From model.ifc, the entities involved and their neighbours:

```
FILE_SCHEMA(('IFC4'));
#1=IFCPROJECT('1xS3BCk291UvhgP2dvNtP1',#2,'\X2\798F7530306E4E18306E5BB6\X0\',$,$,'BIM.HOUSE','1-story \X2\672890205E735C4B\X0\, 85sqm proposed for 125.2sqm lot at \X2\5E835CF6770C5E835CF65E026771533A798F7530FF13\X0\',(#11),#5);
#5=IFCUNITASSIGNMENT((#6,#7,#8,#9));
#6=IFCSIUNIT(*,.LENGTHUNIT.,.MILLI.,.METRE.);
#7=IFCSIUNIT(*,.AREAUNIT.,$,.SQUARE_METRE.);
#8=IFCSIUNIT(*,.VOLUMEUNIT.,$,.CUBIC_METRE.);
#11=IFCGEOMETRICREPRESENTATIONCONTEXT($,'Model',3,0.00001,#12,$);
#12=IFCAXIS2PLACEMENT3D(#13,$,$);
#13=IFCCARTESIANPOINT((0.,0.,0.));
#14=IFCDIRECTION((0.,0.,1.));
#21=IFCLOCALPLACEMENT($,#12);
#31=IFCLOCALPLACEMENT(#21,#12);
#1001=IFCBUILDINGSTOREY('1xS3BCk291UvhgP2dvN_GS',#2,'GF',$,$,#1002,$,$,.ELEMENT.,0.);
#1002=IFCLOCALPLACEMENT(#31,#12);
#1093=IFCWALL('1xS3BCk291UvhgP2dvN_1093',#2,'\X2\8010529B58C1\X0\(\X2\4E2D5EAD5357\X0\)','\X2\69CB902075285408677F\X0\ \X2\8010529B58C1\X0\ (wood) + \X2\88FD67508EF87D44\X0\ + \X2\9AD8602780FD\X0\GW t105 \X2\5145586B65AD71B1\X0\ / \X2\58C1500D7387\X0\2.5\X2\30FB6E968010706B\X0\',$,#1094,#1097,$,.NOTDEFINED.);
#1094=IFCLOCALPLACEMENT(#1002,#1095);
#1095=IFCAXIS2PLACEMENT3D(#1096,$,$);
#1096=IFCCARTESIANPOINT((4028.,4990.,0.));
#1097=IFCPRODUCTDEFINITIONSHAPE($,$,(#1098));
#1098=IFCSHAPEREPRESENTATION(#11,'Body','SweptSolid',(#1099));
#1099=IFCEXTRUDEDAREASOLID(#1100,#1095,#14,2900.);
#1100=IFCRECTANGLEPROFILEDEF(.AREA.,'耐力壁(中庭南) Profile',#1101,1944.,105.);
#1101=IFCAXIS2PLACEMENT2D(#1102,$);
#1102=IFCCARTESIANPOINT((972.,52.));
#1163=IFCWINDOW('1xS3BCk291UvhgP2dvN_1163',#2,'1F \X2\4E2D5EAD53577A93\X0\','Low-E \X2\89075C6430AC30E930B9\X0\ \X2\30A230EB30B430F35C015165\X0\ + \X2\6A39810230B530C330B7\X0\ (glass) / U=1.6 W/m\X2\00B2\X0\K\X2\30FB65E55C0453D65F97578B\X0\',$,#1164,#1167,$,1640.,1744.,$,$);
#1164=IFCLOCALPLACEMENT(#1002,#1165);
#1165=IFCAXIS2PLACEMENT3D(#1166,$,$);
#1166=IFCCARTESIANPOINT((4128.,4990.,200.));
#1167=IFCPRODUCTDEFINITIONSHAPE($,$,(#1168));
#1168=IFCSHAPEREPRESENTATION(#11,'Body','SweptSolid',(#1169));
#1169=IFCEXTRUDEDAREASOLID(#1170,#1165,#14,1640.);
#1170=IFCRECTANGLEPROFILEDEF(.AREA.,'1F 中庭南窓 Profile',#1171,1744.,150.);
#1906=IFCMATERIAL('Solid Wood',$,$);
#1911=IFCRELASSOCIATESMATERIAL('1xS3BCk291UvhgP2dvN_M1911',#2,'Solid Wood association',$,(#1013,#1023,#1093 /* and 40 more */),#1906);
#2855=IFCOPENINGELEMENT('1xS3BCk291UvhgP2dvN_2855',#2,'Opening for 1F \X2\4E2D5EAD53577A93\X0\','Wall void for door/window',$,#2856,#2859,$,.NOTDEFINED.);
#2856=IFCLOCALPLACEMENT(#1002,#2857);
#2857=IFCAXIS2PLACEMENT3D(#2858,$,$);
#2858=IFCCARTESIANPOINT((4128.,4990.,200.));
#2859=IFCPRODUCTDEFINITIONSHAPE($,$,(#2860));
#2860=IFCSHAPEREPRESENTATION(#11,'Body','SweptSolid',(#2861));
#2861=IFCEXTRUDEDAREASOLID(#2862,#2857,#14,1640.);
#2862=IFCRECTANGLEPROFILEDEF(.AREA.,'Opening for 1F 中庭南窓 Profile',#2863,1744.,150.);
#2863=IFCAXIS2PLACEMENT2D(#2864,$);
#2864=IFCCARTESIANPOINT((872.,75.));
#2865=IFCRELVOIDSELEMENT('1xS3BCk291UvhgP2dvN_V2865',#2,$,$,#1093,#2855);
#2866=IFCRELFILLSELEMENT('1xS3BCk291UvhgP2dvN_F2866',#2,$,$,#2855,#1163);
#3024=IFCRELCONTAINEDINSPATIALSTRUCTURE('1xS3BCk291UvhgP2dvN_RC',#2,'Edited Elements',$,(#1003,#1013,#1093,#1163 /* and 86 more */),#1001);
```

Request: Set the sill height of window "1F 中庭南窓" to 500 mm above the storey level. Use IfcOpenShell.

```python
import numpy as np
import ifcopenshell
import ifcopenshell.api.geometry
import ifcopenshell.geom
import ifcopenshell.util.element
import ifcopenshell.util.placement
import ifcopenshell.util.shape
import ifcopenshell.util.unit

model = ifcopenshell.open("model.ifc")
unit_scale = ifcopenshell.util.unit.calculate_unit_scale(model)

window = model.by_guid("1xS3BCk291UvhgP2dvN_1163")
opening = window.FillsVoids[0].RelatingOpeningElement
storey = ifcopenshell.util.element.get_container(window, ifc_class="IfcBuildingStorey")
level = ifcopenshell.util.placement.get_local_placement(storey.ObjectPlacement)[2, 3]

# The opening's origin need not be at the sill, so measure its lowest point.
shape = ifcopenshell.geom.create_shape(ifcopenshell.geom.settings(), opening)
bottom = ifcopenshell.util.shape.get_shape_bottom_elevation(shape, shape.geometry) / unit_scale
dz = level + 0.5 / unit_scale - bottom

shift = np.array([0.0, 0.0, dz])
# The window is not placed relative to its opening, so move both.
for product in (opening, window):
    matrix = ifcopenshell.util.placement.get_local_placement(product.ObjectPlacement)
    matrix[:3, 3] += shift
    ifcopenshell.api.geometry.edit_object_placement(model, product=product, matrix=matrix, is_si=False)

print(f"moved by {dz * unit_scale:+.3f} m")

model.write("model_updated.ifc")
```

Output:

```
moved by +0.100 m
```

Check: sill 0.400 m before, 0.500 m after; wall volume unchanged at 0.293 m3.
